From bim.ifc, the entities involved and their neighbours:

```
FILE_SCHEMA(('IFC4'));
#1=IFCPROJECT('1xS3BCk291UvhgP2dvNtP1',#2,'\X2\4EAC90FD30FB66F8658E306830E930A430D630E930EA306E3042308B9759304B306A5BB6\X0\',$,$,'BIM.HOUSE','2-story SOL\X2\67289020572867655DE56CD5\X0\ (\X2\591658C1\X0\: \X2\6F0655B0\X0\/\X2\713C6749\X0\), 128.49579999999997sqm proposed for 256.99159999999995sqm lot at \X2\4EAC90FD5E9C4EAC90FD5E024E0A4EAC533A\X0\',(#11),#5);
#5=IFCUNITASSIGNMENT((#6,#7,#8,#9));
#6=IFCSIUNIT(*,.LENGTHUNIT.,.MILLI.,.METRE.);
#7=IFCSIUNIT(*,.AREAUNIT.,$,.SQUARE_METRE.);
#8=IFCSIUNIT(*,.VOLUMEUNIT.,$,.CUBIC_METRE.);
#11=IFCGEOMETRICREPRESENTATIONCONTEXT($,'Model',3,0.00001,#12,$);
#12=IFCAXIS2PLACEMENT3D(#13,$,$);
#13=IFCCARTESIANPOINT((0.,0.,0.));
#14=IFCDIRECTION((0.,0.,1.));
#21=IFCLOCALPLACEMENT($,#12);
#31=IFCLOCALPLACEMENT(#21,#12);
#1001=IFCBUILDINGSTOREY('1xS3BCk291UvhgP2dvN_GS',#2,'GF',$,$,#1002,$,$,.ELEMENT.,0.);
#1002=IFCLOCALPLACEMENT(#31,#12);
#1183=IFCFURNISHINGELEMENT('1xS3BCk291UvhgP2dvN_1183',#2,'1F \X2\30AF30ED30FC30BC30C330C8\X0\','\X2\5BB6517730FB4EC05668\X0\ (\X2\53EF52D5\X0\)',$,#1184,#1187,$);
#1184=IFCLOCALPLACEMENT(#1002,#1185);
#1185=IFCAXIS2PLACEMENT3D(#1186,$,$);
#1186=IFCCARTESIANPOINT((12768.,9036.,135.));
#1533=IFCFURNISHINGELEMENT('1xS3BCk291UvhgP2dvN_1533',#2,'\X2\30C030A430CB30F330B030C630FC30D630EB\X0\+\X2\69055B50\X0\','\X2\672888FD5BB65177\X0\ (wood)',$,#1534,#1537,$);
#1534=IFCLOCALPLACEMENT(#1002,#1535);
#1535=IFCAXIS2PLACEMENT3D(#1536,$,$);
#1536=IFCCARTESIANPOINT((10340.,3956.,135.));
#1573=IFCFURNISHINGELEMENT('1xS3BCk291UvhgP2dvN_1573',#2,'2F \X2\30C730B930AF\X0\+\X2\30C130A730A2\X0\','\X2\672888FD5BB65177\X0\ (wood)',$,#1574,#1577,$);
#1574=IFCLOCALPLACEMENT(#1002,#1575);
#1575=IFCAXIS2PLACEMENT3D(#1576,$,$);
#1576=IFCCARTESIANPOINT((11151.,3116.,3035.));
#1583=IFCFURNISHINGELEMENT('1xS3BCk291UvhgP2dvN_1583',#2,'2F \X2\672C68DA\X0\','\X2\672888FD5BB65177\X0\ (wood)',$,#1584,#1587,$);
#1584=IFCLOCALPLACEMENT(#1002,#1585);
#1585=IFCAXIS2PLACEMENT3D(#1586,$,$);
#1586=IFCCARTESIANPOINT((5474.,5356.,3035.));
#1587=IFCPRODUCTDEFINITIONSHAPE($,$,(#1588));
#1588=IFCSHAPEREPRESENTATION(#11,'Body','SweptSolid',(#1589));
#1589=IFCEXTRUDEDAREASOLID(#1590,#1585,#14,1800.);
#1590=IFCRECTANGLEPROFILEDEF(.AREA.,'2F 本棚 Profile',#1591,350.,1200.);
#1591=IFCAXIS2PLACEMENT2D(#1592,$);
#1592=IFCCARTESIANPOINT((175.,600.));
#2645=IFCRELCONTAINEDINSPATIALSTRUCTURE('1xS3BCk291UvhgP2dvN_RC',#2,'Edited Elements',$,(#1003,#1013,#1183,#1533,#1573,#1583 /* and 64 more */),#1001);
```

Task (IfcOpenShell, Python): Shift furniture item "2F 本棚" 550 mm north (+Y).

```python
import ifcopenshell
import ifcopenshell.api.geometry
import ifcopenshell.util.placement

model = ifcopenshell.open("bim.ifc")

item = model.by_guid("1xS3BCk291UvhgP2dvN_1583")
matrix = ifcopenshell.util.placement.get_local_placement(item.ObjectPlacement)
matrix[1, 3] += 550.0
ifcopenshell.api.geometry.edit_object_placement(model, product=item, matrix=matrix, is_si=False)

print(ifcopenshell.util.placement.get_local_placement(item.ObjectPlacement).round(3) + 0.0)

model.write("bim-out.ifc")
```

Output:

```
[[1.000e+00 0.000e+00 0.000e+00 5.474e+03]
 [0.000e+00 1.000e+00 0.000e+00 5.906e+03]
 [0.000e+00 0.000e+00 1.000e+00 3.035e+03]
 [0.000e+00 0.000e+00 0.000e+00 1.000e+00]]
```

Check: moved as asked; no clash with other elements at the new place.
